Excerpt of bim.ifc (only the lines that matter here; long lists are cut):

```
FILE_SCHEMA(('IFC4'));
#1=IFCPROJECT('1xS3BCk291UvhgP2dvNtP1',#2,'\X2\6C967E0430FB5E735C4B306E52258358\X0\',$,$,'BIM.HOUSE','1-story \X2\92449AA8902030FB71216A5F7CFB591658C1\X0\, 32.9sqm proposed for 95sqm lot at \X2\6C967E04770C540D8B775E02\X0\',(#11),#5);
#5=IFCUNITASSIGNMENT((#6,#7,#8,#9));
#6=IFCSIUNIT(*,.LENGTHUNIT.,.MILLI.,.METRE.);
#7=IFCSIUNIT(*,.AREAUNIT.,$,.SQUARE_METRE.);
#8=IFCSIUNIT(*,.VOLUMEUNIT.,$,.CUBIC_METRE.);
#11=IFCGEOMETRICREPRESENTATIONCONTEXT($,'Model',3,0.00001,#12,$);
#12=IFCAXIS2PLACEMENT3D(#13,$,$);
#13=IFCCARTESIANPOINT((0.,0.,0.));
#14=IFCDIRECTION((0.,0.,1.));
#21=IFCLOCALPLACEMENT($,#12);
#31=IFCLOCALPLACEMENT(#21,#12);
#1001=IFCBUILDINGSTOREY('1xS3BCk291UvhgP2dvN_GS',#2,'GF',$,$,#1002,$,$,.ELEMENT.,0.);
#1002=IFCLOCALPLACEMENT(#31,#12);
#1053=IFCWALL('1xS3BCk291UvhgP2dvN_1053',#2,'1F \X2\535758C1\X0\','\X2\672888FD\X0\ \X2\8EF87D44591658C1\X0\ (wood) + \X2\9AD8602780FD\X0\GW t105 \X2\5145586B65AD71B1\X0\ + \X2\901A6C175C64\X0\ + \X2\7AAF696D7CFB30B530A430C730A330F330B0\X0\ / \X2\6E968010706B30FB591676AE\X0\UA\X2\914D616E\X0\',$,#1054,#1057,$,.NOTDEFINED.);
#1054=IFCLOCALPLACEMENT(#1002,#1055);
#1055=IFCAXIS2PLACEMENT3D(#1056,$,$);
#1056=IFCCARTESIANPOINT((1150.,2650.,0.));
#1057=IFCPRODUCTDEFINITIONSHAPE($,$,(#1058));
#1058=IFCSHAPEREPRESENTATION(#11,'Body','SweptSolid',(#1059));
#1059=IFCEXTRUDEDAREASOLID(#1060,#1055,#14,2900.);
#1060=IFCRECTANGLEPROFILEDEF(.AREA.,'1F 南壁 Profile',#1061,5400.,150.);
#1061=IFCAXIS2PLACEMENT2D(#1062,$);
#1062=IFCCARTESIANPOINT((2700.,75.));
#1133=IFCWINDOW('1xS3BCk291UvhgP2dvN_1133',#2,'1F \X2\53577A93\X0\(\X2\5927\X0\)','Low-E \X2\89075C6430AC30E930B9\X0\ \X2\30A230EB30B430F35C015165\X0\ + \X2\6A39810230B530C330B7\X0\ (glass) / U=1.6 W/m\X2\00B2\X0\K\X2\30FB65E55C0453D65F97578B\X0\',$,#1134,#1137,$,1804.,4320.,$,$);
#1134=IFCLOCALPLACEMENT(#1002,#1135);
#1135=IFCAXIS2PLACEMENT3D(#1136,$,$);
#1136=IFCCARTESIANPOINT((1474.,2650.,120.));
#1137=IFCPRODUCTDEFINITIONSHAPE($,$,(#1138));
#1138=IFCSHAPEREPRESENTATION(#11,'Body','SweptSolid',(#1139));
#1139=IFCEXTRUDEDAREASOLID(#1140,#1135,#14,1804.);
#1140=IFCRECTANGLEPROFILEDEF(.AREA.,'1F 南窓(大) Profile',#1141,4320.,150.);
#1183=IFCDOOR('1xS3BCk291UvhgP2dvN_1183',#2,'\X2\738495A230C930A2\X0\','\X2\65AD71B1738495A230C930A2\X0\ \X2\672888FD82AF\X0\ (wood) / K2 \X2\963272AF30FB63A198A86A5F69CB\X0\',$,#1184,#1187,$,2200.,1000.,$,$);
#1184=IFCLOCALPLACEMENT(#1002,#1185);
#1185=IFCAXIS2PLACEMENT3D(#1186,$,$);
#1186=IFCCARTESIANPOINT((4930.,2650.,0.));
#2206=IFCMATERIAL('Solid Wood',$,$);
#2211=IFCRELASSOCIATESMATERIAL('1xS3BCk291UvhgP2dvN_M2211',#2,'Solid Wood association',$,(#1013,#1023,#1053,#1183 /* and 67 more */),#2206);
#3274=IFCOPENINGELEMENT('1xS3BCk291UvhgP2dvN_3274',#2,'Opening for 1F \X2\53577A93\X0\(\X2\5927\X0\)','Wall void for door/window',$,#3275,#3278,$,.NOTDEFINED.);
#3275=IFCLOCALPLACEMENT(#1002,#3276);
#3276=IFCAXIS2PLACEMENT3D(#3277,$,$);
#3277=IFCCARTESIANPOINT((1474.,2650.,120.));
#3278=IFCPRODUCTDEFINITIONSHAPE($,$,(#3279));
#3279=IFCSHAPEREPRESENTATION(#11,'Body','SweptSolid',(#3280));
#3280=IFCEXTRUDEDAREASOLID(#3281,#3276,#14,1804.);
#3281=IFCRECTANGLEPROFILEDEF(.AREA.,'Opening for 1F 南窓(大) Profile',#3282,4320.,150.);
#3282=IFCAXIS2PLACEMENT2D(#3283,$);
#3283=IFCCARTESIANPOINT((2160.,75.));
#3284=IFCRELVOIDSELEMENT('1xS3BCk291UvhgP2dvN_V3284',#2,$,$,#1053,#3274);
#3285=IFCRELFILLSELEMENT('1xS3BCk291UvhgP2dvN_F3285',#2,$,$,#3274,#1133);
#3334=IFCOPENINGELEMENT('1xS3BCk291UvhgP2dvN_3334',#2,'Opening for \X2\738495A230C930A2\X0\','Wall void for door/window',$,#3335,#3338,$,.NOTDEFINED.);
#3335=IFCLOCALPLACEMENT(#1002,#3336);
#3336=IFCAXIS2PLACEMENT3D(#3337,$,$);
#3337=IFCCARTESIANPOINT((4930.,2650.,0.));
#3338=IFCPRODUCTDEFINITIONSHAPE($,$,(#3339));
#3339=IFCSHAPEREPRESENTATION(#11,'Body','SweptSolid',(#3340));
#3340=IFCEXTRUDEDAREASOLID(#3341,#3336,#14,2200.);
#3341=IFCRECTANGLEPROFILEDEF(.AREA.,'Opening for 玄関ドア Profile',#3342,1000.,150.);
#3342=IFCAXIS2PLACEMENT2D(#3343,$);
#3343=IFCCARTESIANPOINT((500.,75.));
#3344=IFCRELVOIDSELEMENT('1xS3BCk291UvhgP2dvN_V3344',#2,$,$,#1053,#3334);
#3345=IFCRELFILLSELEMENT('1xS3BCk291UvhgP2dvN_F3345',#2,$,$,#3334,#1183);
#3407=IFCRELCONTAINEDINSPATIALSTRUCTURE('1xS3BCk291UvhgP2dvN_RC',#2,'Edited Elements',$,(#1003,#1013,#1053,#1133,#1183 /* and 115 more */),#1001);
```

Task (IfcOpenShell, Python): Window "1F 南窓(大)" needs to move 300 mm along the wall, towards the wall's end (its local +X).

```python
import ifcopenshell
import ifcopenshell.api.geometry
import ifcopenshell.util.placement

model = ifcopenshell.open("bim.ifc")

window = model.by_guid("1xS3BCk291UvhgP2dvN_1133")
opening = window.FillsVoids[0].RelatingOpeningElement
wall = opening.VoidsElements[0].RelatingBuildingElement

wall_matrix = ifcopenshell.util.placement.get_local_placement(wall.ObjectPlacement)
shift = wall_matrix[:3, 0] * 300.0
before = ifcopenshell.util.placement.get_local_placement(window.ObjectPlacement)[:3, 3].copy()

# The window is not placed relative to its opening, so move both.
for product in (opening, window):
    matrix = ifcopenshell.util.placement.get_local_placement(product.ObjectPlacement)
    matrix[:3, 3] += shift
    ifcopenshell.api.geometry.edit_object_placement(model, product=product, matrix=matrix, is_si=False)

after = ifcopenshell.util.placement.get_local_placement(window.ObjectPlacement)[:3, 3]
print("window moved by", (after - before).round(3) + 0.0)

model.write("bim-out.ifc")
```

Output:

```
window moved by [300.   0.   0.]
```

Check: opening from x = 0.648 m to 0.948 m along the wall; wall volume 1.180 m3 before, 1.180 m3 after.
